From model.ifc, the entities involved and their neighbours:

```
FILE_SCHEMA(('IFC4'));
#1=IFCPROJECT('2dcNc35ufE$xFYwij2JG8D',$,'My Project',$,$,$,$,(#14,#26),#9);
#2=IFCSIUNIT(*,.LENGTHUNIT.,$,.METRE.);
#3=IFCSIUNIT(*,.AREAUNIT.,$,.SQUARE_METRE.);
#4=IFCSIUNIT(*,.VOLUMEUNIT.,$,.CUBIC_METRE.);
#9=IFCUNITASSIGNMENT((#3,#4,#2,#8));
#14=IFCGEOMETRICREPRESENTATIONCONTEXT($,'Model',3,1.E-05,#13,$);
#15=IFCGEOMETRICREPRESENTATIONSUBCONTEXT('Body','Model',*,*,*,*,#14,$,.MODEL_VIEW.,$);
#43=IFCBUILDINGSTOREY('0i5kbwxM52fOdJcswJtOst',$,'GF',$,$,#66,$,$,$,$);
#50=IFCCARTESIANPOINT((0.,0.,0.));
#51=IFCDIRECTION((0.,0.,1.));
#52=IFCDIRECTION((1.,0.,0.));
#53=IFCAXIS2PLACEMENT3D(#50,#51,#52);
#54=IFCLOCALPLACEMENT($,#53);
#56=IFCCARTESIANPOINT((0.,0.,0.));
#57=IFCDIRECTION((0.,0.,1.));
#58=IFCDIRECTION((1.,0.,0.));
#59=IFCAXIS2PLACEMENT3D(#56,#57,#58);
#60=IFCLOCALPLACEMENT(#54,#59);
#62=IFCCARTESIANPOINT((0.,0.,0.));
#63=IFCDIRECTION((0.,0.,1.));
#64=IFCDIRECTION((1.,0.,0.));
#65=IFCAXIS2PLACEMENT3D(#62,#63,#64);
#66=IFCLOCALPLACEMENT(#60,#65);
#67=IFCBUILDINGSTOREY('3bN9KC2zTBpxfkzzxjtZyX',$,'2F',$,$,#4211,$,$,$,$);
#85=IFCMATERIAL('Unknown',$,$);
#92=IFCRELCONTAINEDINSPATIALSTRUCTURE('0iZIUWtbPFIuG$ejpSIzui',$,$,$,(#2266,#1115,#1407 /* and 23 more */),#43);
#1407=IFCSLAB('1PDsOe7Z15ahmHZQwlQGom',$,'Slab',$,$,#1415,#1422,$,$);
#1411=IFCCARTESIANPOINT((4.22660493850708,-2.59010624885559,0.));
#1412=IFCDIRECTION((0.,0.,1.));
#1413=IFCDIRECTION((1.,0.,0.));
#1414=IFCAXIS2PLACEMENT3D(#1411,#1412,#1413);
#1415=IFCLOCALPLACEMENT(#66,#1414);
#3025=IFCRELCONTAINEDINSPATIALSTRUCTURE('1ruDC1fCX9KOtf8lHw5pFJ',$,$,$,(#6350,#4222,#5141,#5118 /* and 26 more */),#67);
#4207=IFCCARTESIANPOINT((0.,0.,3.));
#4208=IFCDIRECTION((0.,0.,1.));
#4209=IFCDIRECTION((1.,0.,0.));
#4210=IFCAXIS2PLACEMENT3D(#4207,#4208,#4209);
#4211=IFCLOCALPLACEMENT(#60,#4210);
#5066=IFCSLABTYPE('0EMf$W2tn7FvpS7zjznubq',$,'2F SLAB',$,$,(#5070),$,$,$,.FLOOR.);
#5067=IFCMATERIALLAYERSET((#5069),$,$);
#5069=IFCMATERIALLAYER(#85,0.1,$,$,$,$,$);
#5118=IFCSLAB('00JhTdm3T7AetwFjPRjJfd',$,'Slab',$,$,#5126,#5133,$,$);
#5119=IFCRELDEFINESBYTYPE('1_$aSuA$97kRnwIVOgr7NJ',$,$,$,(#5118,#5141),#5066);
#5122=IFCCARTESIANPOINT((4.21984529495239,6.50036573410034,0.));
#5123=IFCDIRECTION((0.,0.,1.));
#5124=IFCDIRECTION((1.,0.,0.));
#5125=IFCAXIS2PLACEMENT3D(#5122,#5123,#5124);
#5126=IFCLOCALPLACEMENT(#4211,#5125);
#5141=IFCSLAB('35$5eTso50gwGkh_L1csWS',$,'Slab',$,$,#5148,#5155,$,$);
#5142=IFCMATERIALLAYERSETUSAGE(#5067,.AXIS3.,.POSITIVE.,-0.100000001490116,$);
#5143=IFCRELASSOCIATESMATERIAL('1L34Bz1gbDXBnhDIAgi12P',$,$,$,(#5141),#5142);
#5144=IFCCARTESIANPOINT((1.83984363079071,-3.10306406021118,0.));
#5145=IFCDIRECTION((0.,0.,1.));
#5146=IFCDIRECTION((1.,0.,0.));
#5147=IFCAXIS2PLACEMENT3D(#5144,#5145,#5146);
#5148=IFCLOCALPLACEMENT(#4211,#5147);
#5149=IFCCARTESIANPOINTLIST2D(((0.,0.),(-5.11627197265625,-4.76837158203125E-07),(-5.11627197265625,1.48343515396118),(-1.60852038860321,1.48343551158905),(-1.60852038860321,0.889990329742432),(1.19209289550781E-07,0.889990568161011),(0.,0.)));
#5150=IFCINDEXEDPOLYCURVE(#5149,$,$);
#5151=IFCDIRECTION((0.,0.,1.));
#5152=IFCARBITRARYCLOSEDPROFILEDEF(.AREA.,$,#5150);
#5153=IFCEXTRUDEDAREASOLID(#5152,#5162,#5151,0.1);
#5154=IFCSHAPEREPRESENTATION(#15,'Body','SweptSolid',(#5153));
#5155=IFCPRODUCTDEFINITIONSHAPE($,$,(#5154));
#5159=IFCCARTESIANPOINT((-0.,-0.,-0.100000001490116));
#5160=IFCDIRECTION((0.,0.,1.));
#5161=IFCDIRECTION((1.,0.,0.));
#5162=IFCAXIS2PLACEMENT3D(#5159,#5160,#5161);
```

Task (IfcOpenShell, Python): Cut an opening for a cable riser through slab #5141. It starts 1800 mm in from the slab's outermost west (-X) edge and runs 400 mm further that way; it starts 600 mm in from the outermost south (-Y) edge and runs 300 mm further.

```python
import numpy as np
import ifcopenshell
import ifcopenshell.api.feature
import ifcopenshell.api.geometry
import ifcopenshell.api.root
import ifcopenshell.geom
import ifcopenshell.util.placement
import ifcopenshell.util.representation
import ifcopenshell.util.shape
import ifcopenshell.util.unit

model = ifcopenshell.open("model.ifc")
unit_scale = ifcopenshell.util.unit.calculate_unit_scale(model)
settings = ifcopenshell.geom.settings()


def volume(element):
    """Net volume in cubic metres, openings subtracted."""
    shape = ifcopenshell.geom.create_shape(settings, element)
    return ifcopenshell.util.shape.get_volume(shape.geometry)


slab = model.by_id(5141)
before = volume(slab)

# Extent in the slab's own axes, in metres. The edges named are its -X and -Y sides.
slab_shape = ifcopenshell.geom.create_shape(settings, slab)
vertices = ifcopenshell.util.shape.get_vertices(slab_shape.geometry)
x_min, y_min, bottom = vertices.min(axis=0)
top = vertices[:, 2].max()

opening = ifcopenshell.api.root.create_entity(model, ifc_class="IfcOpeningElement", name="Cable riser opening", predefined_type="OPENING")
context = ifcopenshell.util.representation.get_context(model, "Model", "Body", "MODEL_VIEW")
width, depth = 0.4, 0.3
outline = [(0.0, 0.0), (width, 0.0), (width, depth), (0.0, depth), (0.0, 0.0)]
# Overshoot both faces by 50 mm so the cut is clean.
shape = ifcopenshell.api.geometry.add_slab_representation(
    model, context=context, depth=top - bottom + 0.1, polyline=outline
)
ifcopenshell.api.geometry.assign_representation(model, product=opening, representation=shape)

matrix = ifcopenshell.util.placement.get_local_placement(slab.ObjectPlacement)
matrix[:, 3] = matrix @ np.append(np.array([x_min + 1.8, y_min + 0.6, bottom - 0.05]) / unit_scale, 1.0)
ifcopenshell.api.geometry.edit_object_placement(model, product=opening, matrix=matrix, is_si=False)
ifcopenshell.api.feature.add_feature(model, feature=opening, element=slab)

after = volume(slab)

print(f"slab volume {before:.3f} -> {after:.3f} m3")

model.write("model_edited.ifc")
```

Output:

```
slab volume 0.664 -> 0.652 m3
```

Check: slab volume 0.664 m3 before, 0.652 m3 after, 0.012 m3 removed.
